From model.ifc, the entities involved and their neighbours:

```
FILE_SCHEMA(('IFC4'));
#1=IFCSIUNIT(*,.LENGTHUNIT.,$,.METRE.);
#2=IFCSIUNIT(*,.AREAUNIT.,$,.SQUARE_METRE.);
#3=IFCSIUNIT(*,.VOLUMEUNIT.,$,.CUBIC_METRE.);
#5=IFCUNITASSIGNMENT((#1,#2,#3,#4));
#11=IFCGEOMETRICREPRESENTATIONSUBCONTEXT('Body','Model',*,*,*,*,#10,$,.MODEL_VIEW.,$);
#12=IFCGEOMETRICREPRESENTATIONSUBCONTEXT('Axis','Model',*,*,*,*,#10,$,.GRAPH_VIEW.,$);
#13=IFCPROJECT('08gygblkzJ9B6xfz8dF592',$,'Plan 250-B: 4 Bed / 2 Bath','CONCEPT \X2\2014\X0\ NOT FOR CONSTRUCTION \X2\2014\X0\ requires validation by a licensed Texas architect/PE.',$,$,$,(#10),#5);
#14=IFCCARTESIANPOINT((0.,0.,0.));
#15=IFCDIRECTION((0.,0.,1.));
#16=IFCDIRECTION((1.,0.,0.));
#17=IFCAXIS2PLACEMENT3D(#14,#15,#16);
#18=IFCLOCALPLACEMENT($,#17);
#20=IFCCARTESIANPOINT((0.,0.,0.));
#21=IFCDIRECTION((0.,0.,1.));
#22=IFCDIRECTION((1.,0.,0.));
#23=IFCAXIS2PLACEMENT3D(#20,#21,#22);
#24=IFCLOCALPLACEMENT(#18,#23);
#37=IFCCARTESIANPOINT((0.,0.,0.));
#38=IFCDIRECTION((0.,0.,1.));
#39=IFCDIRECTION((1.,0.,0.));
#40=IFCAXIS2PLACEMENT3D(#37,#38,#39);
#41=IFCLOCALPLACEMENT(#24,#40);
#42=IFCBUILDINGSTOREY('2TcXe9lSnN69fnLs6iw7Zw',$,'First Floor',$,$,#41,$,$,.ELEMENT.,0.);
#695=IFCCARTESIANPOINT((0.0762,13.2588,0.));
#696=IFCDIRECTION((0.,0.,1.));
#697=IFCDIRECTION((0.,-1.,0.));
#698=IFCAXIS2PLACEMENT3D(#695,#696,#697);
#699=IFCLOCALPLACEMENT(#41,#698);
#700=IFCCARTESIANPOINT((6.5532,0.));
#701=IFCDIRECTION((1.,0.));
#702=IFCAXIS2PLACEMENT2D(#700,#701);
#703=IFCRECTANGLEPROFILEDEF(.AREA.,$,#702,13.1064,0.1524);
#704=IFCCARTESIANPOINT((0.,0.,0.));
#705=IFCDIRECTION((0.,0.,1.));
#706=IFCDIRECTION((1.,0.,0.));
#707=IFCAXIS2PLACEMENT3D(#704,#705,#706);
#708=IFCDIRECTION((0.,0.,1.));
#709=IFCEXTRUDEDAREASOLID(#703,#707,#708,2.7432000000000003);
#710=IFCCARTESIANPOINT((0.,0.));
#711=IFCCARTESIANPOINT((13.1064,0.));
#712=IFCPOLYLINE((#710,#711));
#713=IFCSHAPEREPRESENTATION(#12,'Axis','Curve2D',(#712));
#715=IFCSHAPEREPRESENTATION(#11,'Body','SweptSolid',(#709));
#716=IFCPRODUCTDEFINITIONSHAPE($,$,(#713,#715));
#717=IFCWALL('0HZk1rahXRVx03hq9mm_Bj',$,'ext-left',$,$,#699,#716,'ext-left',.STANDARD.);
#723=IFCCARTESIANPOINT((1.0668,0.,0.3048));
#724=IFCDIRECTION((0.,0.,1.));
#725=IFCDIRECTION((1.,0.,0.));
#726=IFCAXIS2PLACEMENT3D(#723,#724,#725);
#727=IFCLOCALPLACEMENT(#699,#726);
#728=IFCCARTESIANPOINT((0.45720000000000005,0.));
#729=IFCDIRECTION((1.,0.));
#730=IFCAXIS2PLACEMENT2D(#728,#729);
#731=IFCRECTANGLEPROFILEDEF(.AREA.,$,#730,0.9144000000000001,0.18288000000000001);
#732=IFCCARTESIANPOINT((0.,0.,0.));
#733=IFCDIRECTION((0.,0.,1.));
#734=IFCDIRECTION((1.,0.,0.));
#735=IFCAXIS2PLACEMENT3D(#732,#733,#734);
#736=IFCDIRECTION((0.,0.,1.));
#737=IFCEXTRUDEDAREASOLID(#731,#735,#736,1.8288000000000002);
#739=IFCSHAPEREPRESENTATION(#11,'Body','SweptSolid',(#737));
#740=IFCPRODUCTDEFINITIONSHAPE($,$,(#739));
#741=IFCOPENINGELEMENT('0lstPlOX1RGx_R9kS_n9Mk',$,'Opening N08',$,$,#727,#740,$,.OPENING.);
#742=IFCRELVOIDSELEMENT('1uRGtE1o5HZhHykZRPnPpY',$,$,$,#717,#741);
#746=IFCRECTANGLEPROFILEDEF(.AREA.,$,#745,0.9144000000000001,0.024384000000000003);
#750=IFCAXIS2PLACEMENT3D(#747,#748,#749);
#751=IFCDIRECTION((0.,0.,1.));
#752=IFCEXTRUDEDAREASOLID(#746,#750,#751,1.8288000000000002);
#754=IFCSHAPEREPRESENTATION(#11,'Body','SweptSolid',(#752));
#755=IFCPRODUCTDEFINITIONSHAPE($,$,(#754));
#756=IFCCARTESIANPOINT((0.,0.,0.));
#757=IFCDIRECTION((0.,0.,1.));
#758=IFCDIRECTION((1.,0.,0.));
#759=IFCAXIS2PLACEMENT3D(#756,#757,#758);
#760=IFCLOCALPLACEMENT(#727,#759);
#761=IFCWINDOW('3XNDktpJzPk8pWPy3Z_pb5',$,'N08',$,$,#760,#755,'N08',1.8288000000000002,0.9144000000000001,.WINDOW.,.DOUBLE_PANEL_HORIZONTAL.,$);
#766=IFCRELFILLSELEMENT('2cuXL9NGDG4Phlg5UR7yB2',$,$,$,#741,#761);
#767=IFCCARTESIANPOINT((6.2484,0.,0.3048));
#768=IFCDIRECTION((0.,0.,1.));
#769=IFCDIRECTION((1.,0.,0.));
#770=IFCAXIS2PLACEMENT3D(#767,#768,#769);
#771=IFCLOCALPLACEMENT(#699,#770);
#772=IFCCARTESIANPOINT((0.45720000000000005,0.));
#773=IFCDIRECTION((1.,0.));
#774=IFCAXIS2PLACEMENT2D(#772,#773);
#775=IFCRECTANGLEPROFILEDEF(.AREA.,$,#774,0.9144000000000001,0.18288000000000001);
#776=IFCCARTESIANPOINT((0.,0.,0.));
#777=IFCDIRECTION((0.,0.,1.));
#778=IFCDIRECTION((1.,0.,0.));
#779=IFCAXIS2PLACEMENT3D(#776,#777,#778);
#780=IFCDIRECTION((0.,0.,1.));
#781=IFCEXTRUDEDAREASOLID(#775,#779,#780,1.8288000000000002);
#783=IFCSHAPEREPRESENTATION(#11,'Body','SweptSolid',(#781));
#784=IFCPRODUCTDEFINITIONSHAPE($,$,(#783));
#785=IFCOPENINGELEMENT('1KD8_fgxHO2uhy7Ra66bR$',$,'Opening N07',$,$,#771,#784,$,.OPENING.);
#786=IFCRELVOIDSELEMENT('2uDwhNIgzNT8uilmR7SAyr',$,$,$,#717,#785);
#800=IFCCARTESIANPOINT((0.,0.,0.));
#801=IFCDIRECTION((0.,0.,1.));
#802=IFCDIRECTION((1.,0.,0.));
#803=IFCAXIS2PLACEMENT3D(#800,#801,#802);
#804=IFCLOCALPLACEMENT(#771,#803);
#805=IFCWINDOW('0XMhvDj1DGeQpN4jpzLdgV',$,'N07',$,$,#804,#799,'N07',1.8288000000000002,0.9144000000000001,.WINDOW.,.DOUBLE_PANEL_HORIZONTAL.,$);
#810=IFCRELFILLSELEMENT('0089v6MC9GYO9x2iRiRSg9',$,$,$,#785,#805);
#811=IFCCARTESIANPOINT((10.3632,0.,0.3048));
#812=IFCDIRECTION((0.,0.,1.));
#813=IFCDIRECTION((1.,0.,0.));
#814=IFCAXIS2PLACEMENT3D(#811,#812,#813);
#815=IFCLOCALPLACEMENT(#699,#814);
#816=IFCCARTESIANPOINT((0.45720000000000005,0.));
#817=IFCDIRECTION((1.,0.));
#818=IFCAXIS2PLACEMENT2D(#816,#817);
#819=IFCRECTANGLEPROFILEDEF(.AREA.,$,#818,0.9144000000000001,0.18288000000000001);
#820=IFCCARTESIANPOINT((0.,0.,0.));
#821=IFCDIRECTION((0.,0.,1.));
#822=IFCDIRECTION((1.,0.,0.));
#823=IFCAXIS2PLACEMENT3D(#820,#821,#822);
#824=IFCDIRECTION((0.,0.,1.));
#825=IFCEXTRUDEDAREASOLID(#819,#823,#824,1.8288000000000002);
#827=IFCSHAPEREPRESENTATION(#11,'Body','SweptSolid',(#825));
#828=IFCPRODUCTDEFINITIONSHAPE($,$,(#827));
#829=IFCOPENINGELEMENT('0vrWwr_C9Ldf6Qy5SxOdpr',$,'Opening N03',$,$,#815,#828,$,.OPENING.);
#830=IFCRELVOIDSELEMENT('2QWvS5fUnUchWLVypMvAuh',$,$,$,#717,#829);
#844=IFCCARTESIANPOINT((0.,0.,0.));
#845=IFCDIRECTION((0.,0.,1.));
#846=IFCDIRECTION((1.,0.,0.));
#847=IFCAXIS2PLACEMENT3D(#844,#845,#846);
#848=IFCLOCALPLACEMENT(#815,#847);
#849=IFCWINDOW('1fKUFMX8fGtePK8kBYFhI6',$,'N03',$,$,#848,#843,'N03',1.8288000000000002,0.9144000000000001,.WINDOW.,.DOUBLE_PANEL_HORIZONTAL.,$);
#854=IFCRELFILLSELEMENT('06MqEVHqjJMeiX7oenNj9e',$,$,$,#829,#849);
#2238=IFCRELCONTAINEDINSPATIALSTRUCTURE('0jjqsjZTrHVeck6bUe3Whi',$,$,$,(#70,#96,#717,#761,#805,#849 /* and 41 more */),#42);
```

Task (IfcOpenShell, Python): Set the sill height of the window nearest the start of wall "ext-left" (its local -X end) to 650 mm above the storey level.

```python
import numpy as np
import ifcopenshell
import ifcopenshell.api.geometry
import ifcopenshell.geom
import ifcopenshell.util.element
import ifcopenshell.util.placement
import ifcopenshell.util.shape
import ifcopenshell.util.unit

model = ifcopenshell.open("model.ifc")
unit_scale = ifcopenshell.util.unit.calculate_unit_scale(model)

window = model.by_id(761)
opening = window.FillsVoids[0].RelatingOpeningElement
storey = ifcopenshell.util.element.get_container(window, ifc_class="IfcBuildingStorey")
level = ifcopenshell.util.placement.get_local_placement(storey.ObjectPlacement)[2, 3]

# The opening's origin need not be at the sill, so measure its lowest point.
shape = ifcopenshell.geom.create_shape(ifcopenshell.geom.settings(), opening)
bottom = ifcopenshell.util.shape.get_shape_bottom_elevation(shape, shape.geometry) / unit_scale
dz = level + 0.65 - bottom

shift = np.array([0.0, 0.0, dz])
# The window is placed relative to its opening, so it follows when the opening moves.
matrix = ifcopenshell.util.placement.get_local_placement(opening.ObjectPlacement)
matrix[:3, 3] += shift
ifcopenshell.api.geometry.edit_object_placement(
    model, product=opening, matrix=matrix, is_si=False, should_transform_children=True
)

print(f"moved by {dz * unit_scale:+.3f} m")

model.write("model_edited.ifc")
```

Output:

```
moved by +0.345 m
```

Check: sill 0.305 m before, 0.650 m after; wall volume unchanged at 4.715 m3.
